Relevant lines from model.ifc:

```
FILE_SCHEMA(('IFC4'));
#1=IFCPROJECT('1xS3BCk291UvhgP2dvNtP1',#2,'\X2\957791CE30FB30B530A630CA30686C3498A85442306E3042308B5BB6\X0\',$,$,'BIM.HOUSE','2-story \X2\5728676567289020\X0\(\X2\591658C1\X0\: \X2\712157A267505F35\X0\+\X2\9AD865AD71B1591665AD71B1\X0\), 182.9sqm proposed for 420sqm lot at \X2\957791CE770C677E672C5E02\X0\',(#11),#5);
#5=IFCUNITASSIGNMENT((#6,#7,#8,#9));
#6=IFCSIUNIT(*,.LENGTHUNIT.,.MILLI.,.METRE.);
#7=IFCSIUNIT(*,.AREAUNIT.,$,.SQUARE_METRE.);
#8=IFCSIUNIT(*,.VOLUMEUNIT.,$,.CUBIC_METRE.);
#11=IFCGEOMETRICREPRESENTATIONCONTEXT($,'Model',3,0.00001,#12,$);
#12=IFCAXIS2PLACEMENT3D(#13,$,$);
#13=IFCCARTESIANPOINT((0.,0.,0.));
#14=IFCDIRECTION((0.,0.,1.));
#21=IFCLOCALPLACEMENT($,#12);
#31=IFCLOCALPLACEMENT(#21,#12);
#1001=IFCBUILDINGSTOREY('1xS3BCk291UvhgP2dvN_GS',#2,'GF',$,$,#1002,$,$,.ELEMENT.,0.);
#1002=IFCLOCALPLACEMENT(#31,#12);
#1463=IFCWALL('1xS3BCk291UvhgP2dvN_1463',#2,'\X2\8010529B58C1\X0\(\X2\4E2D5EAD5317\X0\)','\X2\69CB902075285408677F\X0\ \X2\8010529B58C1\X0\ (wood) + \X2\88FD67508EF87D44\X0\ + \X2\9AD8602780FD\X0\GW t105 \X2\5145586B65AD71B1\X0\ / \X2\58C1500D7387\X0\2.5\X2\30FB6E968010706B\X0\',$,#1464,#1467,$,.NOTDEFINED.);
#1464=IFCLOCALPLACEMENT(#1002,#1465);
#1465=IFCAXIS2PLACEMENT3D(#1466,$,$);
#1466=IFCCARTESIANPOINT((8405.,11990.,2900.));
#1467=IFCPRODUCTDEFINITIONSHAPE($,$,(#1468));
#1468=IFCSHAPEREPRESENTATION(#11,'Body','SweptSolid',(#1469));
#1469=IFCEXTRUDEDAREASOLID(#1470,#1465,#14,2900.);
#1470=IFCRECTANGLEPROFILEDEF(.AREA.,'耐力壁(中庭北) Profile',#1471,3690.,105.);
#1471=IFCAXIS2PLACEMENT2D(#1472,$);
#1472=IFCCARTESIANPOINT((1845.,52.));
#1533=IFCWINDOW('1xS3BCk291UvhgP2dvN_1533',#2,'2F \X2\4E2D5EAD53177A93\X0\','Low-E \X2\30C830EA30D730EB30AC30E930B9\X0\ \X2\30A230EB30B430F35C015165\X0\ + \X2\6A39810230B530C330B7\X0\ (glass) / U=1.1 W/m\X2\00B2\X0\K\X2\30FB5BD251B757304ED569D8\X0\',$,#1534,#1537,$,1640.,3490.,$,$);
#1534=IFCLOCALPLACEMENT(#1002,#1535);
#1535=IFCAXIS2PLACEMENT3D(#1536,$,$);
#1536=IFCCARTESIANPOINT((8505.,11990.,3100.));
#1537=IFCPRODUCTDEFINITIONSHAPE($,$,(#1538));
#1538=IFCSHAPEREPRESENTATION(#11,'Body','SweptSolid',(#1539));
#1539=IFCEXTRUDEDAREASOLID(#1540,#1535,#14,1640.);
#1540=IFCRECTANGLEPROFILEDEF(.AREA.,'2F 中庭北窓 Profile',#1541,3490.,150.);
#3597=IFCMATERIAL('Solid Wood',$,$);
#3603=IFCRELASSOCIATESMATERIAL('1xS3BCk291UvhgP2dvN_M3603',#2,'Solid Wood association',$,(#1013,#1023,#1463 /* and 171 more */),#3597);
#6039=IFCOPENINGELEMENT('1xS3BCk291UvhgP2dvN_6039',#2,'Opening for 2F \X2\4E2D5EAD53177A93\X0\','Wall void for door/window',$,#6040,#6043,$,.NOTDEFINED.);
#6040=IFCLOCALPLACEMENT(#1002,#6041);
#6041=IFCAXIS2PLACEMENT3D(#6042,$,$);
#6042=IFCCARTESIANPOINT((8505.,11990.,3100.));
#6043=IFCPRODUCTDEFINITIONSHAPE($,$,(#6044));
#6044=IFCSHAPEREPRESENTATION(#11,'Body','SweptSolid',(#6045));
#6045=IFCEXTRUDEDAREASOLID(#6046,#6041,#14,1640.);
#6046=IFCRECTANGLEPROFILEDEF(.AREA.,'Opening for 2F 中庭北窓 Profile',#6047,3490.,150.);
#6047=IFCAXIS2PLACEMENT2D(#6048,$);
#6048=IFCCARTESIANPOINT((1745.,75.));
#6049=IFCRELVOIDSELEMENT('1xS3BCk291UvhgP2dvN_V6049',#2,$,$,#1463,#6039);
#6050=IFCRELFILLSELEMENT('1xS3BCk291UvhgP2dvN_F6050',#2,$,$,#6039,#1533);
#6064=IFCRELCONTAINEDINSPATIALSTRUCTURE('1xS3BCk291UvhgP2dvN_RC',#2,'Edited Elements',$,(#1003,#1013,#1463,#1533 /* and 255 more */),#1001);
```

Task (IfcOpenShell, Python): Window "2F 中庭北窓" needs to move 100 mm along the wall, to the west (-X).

```python
import ifcopenshell
import ifcopenshell.api.geometry
import ifcopenshell.util.placement

model = ifcopenshell.open("model.ifc")

window = model.by_guid("1xS3BCk291UvhgP2dvN_1533")
opening = window.FillsVoids[0].RelatingOpeningElement
wall = opening.VoidsElements[0].RelatingBuildingElement

wall_matrix = ifcopenshell.util.placement.get_local_placement(wall.ObjectPlacement)
shift = wall_matrix[:3, 0] * -100.0
before = ifcopenshell.util.placement.get_local_placement(window.ObjectPlacement)[:3, 3].copy()

# The window is not placed relative to its opening, so move both.
for product in (opening, window):
    matrix = ifcopenshell.util.placement.get_local_placement(product.ObjectPlacement)
    matrix[:3, 3] += shift
    ifcopenshell.api.geometry.edit_object_placement(model, product=product, matrix=matrix, is_si=False)

after = ifcopenshell.util.placement.get_local_placement(window.ObjectPlacement)[:3, 3]
print("window moved by", (after - before).round(3) + 0.0)

model.write("model-out.ifc")
```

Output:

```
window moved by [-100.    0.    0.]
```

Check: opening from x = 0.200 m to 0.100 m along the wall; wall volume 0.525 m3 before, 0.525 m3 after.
